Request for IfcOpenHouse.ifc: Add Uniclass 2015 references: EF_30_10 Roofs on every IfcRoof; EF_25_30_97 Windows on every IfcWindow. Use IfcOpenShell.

First a look at what the model holds.

```python
import ifcopenshell

model = ifcopenshell.open("IfcOpenHouse.ifc")
print(model.schema)
print("classifications:", [c.Name for c in model.by_type("IfcClassification")])
for ifc_class in ("IfcDoor", "IfcRoof", "IfcStair", "IfcWall", "IfcWindow"):
    print(ifc_class, len(model.by_type(ifc_class)))
```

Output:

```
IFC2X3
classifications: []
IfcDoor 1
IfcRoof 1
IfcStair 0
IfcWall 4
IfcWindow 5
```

```python
import ifcopenshell
import ifcopenshell.api.classification

model = ifcopenshell.open("IfcOpenHouse.ifc")

# IFC2X3 requires Source and Edition and has no link from the project to the system.
system = model.create_entity("IfcClassification", Source="NBS", Edition="2015", Name="Uniclass 2015")

codes = {
    "IfcRoof": ("EF_30_10", "Roofs"),
    "IfcWindow": ("EF_25_30_97", "Windows"),
}
for ifc_class, (code, name) in codes.items():
    products = model.by_type(ifc_class)
    ifcopenshell.api.classification.add_reference(
        model, products=products, classification=system, identification=code, name=name
    )
    print(code, len(products))

model.write("IfcOpenHouse_rev.ifc")
```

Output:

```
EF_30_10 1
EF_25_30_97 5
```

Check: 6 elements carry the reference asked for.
